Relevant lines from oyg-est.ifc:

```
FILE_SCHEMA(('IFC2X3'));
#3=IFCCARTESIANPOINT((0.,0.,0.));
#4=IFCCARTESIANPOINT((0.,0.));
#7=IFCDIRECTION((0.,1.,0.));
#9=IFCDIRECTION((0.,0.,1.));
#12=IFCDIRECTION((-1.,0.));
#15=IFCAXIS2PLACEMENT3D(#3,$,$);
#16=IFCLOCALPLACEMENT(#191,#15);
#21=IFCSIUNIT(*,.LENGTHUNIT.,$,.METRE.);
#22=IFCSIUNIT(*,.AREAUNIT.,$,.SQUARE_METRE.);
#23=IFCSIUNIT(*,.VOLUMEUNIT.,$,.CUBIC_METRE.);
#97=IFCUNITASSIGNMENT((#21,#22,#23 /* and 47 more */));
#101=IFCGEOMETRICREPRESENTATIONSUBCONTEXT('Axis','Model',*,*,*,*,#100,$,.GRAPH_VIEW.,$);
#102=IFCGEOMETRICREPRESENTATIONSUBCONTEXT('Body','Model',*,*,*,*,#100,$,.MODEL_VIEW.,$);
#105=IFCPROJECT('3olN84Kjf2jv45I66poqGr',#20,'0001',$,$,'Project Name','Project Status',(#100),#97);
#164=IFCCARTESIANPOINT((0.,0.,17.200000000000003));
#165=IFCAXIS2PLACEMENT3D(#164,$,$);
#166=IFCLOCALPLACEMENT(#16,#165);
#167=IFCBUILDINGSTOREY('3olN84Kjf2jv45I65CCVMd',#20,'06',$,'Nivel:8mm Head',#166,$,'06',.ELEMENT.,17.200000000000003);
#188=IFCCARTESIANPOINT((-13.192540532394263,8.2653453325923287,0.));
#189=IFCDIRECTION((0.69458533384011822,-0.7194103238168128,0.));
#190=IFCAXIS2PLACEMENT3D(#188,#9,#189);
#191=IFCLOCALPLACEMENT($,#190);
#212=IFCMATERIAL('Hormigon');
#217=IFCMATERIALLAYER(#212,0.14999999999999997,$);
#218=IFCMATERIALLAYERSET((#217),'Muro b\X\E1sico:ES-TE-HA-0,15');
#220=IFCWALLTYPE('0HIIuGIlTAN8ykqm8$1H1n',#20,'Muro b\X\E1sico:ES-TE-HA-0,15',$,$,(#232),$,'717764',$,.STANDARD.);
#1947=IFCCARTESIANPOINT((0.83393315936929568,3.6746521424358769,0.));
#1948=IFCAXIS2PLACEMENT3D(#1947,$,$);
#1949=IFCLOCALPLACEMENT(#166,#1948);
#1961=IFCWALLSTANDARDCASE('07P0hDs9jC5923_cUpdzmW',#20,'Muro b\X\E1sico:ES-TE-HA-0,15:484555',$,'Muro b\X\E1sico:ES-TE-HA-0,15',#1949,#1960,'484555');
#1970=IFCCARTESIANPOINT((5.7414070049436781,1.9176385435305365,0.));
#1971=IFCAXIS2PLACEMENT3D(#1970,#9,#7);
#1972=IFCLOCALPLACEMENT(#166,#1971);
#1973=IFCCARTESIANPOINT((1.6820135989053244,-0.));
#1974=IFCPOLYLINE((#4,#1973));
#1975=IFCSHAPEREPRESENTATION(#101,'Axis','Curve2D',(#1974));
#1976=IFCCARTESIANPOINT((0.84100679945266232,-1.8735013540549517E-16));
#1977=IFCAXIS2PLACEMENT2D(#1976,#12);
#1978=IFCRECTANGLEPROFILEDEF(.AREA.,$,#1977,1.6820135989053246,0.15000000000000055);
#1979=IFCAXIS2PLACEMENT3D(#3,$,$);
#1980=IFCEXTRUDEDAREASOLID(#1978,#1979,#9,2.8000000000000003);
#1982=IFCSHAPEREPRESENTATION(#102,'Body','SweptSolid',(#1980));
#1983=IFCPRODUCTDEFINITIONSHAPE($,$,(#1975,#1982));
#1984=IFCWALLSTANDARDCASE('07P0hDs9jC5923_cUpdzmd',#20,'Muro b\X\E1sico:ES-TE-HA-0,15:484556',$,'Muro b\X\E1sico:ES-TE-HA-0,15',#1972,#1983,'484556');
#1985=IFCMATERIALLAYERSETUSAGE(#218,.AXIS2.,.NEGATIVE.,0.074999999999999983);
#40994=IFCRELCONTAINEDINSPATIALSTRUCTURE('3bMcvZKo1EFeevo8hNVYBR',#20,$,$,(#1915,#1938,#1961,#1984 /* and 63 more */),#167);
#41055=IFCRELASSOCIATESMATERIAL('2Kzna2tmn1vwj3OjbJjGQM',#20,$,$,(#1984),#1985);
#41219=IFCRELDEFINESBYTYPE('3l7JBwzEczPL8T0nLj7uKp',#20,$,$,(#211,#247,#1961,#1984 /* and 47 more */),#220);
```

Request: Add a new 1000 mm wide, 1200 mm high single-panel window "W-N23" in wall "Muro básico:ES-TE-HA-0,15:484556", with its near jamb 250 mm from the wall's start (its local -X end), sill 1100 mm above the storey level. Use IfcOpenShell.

```python
import numpy as np
import ifcopenshell
import ifcopenshell.api.feature
import ifcopenshell.api.geometry
import ifcopenshell.api.root
import ifcopenshell.api.spatial
import ifcopenshell.api.type
import ifcopenshell.geom
import ifcopenshell.util.element
import ifcopenshell.util.placement
import ifcopenshell.util.representation
import ifcopenshell.util.shape
import ifcopenshell.util.unit

model = ifcopenshell.open("oyg-est.ifc")
unit_scale = ifcopenshell.util.unit.calculate_unit_scale(model)
settings = ifcopenshell.geom.settings()


def volume(element):
    """Net volume in cubic metres, openings subtracted."""
    shape = ifcopenshell.geom.create_shape(settings, element)
    return ifcopenshell.util.shape.get_volume(shape.geometry)


wall = model.by_id(1984)
storey = ifcopenshell.util.element.get_container(wall, ifc_class="IfcBuildingStorey")
context = ifcopenshell.util.representation.get_context(model, "Model", "Body", "MODEL_VIEW")
before = volume(wall)

width, height, from_end, sill = 1, 1.2, 0.25, 1.1  # metres

# The wall runs along its own X axis, and the end named is its -X end.
wall_shape = ifcopenshell.geom.create_shape(settings, wall)
x, y, z = ifcopenshell.util.shape.get_vertices(wall_shape.geometry).T
start = x.min() + from_end
face, thickness = float(y.min()), float(y.max() - y.min())
wall_matrix = ifcopenshell.util.placement.get_local_placement(wall.ObjectPlacement)
level = ifcopenshell.util.placement.get_local_placement(storey.ObjectPlacement)[2, 3]


def in_wall(x, y):
    """Placement at x, y metres in the wall's axes, at sill height."""
    matrix = wall_matrix.copy()
    matrix[:, 3] = wall_matrix @ np.array([x / unit_scale, y / unit_scale, 0.0, 1.0])
    matrix[2, 3] = level + sill / unit_scale
    return matrix


# Opening: a box that overshoots both wall faces by 50 mm.
opening = ifcopenshell.api.root.create_entity(model, ifc_class="IfcOpeningElement")
box = ifcopenshell.api.geometry.add_wall_representation(
    model, context=context, length=width, height=height, thickness=thickness + 0.1
)
ifcopenshell.api.geometry.assign_representation(model, product=opening, representation=box)
ifcopenshell.api.geometry.edit_object_placement(model, product=opening, matrix=in_wall(start, face - 0.05), is_si=False)
ifcopenshell.api.feature.add_feature(model, feature=opening, element=wall)

window = ifcopenshell.api.root.create_entity(model, ifc_class="IfcWindow", name="W-N23")
window.OverallWidth, window.OverallHeight = width / unit_scale, height / unit_scale
body = ifcopenshell.api.geometry.add_window_representation(
    model,
    context=context,
    overall_width=window.OverallWidth,
    overall_height=window.OverallHeight,
    partition_type="SINGLE_PANEL",
)
ifcopenshell.api.geometry.assign_representation(model, product=window, representation=body)
ifcopenshell.api.spatial.assign_container(model, products=[window], relating_structure=storey)
fills = ifcopenshell.api.feature.add_filling(model, opening=opening, element=window)
fills.OwnerHistory = window.OwnerHistory  # required in IFC2X3

# IFC2X3 keeps the operation on the window style.
style = ifcopenshell.api.root.create_entity(model, ifc_class="IfcWindowStyle", name="W-N23")
style.OperationType, style.ConstructionType = "SINGLE_PANEL", "NOTDEFINED"
style.ParameterTakesPrecedence = style.Sizeable = False
ifcopenshell.api.type.assign_type(model, related_objects=[window], relating_type=style)

# Centre the window in the wall's thickness.
ifcopenshell.api.geometry.edit_object_placement(model, product=window, matrix=in_wall(start, face), is_si=False)
window_shape = ifcopenshell.geom.create_shape(settings, window)
depth = ifcopenshell.util.shape.get_vertices(window_shape.geometry)[:, 1]
offset = face + thickness / 2 - (depth.min() + depth.max()) / 2
ifcopenshell.api.geometry.edit_object_placement(model, product=window, matrix=in_wall(start, offset), is_si=False)

after = volume(wall)

print(f"wall volume {before:.3f} -> {after:.3f} m3")

model.write("oyg-est_v2.ifc")
```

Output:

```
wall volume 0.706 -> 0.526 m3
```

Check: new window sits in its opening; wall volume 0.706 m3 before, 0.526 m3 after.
